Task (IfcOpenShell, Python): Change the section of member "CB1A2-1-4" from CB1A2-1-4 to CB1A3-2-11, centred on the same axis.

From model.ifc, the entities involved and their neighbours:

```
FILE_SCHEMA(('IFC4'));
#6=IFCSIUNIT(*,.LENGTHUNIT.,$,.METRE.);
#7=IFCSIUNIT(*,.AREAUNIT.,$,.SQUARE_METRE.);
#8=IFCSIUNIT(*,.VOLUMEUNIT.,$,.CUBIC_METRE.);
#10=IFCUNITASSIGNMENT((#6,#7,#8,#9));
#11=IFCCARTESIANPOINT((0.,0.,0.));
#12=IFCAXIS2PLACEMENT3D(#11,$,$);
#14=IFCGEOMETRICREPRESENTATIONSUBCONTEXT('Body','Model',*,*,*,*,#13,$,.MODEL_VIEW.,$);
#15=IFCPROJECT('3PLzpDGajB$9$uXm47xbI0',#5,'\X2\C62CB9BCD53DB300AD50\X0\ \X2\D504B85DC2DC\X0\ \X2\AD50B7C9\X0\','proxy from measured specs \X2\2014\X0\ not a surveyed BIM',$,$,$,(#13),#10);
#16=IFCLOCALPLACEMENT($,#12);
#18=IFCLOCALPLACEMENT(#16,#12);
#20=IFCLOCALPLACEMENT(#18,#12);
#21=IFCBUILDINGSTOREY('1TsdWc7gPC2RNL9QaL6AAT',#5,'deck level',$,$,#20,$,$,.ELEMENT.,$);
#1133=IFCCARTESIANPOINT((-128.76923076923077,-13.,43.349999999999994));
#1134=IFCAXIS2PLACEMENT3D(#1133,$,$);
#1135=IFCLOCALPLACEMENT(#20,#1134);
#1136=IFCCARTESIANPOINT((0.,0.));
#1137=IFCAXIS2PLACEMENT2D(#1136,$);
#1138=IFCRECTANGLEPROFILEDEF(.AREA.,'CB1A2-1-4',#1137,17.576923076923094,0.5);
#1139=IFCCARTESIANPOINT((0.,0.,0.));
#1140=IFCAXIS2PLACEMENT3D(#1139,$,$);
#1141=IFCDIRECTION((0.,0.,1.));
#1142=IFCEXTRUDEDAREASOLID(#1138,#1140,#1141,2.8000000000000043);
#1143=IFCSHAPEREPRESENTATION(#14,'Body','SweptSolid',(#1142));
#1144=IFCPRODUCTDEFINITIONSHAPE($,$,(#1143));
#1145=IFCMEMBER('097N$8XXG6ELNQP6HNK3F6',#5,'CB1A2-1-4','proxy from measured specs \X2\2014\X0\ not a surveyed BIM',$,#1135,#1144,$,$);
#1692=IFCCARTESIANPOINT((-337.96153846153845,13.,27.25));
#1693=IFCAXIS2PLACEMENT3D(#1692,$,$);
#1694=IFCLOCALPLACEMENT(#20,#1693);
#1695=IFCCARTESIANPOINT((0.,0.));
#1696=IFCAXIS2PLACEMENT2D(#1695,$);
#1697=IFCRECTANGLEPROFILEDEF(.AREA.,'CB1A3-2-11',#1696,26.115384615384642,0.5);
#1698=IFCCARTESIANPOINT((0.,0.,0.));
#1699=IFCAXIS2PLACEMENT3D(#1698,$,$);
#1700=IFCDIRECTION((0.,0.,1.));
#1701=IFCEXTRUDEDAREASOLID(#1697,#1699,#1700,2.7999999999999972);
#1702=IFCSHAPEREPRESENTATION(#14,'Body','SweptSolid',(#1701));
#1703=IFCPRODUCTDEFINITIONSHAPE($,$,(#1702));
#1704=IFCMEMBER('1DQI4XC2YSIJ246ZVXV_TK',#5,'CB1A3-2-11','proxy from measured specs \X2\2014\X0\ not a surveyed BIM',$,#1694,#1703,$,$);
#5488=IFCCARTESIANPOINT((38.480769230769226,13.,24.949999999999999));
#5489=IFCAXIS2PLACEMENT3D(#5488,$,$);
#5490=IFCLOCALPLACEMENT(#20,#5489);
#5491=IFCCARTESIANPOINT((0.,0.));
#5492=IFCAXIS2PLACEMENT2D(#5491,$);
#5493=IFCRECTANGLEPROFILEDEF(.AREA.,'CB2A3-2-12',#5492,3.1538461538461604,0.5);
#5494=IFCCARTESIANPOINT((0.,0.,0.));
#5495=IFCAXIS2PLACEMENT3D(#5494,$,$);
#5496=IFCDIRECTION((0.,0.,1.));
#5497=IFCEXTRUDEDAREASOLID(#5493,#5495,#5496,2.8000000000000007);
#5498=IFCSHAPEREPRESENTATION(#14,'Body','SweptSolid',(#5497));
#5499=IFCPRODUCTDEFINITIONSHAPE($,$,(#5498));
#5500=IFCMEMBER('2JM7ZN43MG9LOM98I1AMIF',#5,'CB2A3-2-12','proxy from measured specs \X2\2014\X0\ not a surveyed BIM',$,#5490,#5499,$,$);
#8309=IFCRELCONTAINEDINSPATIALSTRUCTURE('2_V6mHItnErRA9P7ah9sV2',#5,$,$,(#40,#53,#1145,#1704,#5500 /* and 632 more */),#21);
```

```python
import ifcopenshell
import ifcopenshell.util.element
import ifcopenshell.util.representation

model = ifcopenshell.open("model.ifc")

member = model.by_id(1145)
source = next(p for p in model.by_type("IfcRectangleProfileDef") if p.ProfileName == "CB1A3-2-11")

body = ifcopenshell.util.representation.get_representation(member, "Model", "Body")
solid = body.Items[0]
old_profile = solid.SweptArea

# Copy the section's sizes but keep this member's own profile position.
profile = ifcopenshell.util.element.copy(model, source)
profile.Position = old_profile.Position
solid.SweptArea = profile
if not model.get_total_inverses(old_profile):
    ifcopenshell.util.element.remove_deep2(model, old_profile)
member.Name = member.Name.replace("CB1A2-1-4", "CB1A3-2-11")

print(solid.SweptArea)

model.write("model_rev.ifc")
```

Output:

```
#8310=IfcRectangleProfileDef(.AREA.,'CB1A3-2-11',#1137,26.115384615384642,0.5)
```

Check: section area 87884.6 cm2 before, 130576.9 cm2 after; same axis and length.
